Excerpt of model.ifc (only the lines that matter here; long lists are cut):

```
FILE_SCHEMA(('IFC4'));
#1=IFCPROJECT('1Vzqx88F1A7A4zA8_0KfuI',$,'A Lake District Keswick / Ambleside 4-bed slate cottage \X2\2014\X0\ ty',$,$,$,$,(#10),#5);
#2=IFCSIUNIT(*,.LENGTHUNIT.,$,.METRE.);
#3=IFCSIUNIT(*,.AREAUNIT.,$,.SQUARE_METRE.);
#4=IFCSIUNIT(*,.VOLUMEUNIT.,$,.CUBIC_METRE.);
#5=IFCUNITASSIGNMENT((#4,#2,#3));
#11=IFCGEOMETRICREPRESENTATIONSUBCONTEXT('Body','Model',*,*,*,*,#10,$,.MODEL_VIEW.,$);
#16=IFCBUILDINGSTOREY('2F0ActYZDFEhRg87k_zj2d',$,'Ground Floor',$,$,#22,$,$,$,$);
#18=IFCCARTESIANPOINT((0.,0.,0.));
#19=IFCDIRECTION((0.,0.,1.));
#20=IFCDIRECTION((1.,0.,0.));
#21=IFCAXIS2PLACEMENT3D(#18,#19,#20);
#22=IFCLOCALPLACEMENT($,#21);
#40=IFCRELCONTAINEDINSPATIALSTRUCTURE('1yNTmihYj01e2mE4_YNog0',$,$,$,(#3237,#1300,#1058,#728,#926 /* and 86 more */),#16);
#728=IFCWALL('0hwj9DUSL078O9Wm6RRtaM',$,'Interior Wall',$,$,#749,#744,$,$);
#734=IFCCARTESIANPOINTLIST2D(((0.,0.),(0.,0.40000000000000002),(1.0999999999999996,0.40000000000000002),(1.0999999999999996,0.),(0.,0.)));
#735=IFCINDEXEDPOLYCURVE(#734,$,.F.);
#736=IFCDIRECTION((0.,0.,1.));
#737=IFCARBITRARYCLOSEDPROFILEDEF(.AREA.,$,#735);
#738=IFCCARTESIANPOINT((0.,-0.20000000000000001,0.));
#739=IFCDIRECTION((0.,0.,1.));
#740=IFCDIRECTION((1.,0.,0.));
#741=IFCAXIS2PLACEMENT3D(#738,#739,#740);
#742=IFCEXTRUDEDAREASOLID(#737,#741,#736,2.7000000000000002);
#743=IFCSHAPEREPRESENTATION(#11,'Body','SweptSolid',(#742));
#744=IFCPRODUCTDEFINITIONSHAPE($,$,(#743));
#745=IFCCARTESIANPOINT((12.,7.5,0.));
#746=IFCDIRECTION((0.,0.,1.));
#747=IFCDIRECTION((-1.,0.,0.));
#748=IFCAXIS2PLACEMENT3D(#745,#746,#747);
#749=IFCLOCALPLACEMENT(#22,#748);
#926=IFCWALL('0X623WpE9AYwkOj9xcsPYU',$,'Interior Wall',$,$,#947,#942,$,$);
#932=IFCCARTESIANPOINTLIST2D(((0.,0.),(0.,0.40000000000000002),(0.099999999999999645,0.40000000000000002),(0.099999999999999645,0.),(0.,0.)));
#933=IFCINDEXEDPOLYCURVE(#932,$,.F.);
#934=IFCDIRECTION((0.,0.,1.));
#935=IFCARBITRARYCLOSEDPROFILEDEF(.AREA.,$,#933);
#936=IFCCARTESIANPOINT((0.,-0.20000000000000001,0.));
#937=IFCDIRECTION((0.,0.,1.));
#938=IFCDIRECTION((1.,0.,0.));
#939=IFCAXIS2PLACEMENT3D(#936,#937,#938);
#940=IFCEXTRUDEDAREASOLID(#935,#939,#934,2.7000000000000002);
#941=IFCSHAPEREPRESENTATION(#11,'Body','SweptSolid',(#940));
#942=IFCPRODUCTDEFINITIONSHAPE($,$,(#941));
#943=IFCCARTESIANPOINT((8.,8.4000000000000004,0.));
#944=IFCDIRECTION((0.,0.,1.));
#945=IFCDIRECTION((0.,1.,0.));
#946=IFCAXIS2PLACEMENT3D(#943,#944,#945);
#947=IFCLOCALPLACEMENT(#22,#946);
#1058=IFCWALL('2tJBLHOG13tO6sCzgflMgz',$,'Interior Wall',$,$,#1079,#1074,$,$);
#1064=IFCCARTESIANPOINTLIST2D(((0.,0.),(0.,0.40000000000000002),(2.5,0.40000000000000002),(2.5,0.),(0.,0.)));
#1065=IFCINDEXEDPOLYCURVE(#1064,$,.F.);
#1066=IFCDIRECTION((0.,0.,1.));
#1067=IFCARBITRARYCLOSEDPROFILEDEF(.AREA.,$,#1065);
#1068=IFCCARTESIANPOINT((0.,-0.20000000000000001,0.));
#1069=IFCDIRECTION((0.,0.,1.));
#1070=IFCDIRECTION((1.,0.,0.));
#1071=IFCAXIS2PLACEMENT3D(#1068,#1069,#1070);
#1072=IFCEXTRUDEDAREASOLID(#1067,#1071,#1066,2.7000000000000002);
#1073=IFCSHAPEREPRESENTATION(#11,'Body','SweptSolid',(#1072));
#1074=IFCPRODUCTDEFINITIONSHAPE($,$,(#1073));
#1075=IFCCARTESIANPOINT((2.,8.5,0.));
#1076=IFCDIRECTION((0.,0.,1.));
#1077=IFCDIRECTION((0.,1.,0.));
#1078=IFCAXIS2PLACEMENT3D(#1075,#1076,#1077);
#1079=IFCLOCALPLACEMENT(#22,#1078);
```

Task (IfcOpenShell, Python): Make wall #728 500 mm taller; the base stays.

```python
import ifcopenshell
import ifcopenshell.geom
import ifcopenshell.util.representation
import ifcopenshell.util.shape
import ifcopenshell.util.unit

model = ifcopenshell.open("model.ifc")
unit_scale = ifcopenshell.util.unit.calculate_unit_scale(model)
settings = ifcopenshell.geom.settings()


def volume(element):
    """Net volume in cubic metres, openings subtracted."""
    shape = ifcopenshell.geom.create_shape(settings, element)
    return ifcopenshell.util.shape.get_volume(shape.geometry)


wall = model.by_id(728)
before = volume(wall)

body = ifcopenshell.util.representation.get_representation(wall, "Model", "Body")
solid = body.Items[0]
old_height = solid.Depth
solid.Depth += 0.5 / unit_scale
after = volume(wall)

print(f"height {old_height:g} -> {solid.Depth:g}, volume {before:.3f} -> {after:.3f} m3")

model.write("model_updated.ifc")
```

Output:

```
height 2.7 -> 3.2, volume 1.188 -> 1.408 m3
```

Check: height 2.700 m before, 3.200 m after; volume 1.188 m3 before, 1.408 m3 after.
